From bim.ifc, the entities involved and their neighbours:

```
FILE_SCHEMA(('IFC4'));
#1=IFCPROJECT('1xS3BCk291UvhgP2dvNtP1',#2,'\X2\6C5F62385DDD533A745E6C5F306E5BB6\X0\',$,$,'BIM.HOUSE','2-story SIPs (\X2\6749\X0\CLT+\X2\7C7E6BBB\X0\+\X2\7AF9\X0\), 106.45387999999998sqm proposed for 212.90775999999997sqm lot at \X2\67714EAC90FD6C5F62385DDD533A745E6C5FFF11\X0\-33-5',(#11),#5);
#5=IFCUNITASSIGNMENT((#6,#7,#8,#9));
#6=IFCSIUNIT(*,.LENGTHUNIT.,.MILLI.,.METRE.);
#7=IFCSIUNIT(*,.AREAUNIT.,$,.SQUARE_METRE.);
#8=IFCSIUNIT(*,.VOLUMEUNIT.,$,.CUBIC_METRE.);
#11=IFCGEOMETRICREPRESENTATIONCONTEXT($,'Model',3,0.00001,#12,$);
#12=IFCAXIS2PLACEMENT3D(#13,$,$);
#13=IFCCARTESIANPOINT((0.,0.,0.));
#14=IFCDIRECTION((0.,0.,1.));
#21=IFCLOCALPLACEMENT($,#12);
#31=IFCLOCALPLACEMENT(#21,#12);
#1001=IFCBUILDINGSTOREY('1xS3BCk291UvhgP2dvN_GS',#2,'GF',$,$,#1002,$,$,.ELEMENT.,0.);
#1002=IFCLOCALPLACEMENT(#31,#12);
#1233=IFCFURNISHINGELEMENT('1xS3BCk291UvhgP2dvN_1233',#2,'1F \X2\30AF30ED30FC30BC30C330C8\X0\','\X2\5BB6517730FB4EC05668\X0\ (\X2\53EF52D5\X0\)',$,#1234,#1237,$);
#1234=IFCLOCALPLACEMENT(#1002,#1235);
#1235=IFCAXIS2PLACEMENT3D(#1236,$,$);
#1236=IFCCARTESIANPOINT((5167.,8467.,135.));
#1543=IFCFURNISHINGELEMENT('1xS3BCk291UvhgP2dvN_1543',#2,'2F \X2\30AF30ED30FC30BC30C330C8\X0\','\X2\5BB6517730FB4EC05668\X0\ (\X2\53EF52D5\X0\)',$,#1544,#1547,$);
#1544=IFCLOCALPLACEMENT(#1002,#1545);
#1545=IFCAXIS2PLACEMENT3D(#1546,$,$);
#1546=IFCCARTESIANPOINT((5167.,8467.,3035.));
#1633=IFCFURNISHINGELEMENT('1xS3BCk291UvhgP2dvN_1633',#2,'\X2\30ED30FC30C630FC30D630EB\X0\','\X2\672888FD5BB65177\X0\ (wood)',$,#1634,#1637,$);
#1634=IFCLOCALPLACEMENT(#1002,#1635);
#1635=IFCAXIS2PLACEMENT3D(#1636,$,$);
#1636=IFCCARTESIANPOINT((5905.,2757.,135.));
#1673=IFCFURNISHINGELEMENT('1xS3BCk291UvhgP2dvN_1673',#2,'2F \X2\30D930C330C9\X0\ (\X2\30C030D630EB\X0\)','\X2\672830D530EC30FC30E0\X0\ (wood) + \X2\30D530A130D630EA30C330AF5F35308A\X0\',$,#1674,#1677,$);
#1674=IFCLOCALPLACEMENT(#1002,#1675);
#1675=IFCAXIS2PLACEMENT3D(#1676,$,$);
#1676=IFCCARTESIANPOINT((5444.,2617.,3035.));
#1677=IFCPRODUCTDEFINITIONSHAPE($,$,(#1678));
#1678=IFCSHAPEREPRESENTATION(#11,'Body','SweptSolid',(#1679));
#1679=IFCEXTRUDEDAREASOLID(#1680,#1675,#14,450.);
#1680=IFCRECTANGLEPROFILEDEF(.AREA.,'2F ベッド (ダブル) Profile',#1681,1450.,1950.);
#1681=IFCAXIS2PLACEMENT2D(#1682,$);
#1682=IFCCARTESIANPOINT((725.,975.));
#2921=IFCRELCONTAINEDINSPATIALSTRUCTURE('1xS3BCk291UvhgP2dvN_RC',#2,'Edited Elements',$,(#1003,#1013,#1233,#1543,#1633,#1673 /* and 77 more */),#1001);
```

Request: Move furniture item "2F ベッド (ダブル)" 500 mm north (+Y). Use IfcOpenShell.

```python
import ifcopenshell
import ifcopenshell.api.geometry
import ifcopenshell.util.placement

model = ifcopenshell.open("bim.ifc")

item = model.by_id(1673)
matrix = ifcopenshell.util.placement.get_local_placement(item.ObjectPlacement)
matrix[1, 3] += 500.0
ifcopenshell.api.geometry.edit_object_placement(model, product=item, matrix=matrix, is_si=False)

print(ifcopenshell.util.placement.get_local_placement(item.ObjectPlacement).round(3) + 0.0)

model.write("bim_rev.ifc")
```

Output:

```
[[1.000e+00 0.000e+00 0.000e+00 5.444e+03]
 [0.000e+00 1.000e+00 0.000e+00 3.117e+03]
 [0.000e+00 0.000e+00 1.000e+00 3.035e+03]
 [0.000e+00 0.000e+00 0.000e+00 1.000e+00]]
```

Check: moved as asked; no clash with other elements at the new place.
